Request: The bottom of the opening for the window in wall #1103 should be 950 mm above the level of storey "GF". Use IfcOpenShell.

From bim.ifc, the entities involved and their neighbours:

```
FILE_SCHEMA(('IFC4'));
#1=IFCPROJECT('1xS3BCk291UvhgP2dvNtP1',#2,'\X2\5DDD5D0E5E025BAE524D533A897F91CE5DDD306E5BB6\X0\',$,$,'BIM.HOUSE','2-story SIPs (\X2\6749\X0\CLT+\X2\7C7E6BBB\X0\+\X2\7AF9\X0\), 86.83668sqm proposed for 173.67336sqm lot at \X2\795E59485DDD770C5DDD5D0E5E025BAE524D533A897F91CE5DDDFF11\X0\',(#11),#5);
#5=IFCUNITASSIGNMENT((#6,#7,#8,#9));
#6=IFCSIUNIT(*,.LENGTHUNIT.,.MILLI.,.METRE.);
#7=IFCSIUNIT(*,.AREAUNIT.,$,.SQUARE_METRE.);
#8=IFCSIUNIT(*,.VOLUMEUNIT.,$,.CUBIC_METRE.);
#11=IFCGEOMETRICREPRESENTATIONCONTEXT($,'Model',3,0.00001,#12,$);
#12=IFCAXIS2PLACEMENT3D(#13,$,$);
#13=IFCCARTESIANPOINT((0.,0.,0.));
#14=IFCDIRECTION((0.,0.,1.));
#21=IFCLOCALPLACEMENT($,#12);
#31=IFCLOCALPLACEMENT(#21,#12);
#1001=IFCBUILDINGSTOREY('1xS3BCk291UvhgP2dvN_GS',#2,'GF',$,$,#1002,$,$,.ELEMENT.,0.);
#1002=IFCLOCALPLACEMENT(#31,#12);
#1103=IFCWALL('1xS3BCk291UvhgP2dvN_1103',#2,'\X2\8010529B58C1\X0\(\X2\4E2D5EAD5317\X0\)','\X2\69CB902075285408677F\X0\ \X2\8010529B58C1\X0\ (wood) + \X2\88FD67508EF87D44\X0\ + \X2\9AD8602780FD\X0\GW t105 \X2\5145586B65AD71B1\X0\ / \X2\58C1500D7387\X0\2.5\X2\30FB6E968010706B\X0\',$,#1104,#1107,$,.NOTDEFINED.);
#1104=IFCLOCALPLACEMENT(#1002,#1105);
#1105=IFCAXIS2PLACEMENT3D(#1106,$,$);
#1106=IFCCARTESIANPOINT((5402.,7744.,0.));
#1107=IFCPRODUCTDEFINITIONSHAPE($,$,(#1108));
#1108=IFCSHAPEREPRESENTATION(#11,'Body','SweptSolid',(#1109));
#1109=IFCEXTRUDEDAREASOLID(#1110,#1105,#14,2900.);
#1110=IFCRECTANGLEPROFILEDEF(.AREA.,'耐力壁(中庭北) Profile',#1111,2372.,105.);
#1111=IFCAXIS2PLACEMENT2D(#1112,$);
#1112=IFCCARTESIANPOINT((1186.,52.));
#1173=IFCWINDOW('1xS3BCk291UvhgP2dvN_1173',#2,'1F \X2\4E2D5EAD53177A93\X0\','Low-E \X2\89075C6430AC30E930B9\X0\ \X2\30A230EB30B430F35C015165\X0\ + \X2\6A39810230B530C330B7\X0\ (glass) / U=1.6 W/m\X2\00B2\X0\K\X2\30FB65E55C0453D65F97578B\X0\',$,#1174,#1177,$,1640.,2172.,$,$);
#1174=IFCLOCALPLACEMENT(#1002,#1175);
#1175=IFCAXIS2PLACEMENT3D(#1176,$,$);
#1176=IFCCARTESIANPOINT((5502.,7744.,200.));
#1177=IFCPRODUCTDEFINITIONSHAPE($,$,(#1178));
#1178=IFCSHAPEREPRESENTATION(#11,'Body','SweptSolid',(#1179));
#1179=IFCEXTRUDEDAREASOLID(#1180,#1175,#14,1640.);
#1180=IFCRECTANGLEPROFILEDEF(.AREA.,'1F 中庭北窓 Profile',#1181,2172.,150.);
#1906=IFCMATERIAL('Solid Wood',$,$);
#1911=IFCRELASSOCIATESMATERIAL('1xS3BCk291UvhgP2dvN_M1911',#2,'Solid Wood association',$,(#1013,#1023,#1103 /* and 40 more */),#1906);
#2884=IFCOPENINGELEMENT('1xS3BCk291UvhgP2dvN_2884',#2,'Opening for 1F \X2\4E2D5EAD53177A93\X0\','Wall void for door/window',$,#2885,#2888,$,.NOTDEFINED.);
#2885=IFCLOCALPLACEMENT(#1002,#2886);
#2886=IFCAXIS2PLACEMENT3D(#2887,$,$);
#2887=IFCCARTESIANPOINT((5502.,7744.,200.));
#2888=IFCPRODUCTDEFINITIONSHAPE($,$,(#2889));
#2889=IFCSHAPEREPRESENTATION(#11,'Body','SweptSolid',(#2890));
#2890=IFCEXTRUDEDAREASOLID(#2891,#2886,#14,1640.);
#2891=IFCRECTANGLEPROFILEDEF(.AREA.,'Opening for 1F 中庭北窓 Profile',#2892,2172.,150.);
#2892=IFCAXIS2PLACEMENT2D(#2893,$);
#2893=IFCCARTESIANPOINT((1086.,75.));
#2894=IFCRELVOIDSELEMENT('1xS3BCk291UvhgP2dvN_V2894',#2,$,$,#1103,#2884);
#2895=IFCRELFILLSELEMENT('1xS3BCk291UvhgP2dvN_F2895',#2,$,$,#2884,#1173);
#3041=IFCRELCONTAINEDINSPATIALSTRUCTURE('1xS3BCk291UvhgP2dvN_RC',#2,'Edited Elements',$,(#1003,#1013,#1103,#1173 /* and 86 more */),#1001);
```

```python
import numpy as np
import ifcopenshell
import ifcopenshell.api.geometry
import ifcopenshell.geom
import ifcopenshell.util.element
import ifcopenshell.util.placement
import ifcopenshell.util.shape
import ifcopenshell.util.unit

model = ifcopenshell.open("bim.ifc")
unit_scale = ifcopenshell.util.unit.calculate_unit_scale(model)

window = model.by_guid("1xS3BCk291UvhgP2dvN_1173")
opening = window.FillsVoids[0].RelatingOpeningElement
storey = ifcopenshell.util.element.get_container(window, ifc_class="IfcBuildingStorey")
level = ifcopenshell.util.placement.get_local_placement(storey.ObjectPlacement)[2, 3]

# The opening's origin need not be at the sill, so measure its lowest point.
shape = ifcopenshell.geom.create_shape(ifcopenshell.geom.settings(), opening)
bottom = ifcopenshell.util.shape.get_shape_bottom_elevation(shape, shape.geometry) / unit_scale
dz = level + 0.95 / unit_scale - bottom

shift = np.array([0.0, 0.0, dz])
# The window is not placed relative to its opening, so move both.
for product in (opening, window):
    matrix = ifcopenshell.util.placement.get_local_placement(product.ObjectPlacement)
    matrix[:3, 3] += shift
    ifcopenshell.api.geometry.edit_object_placement(model, product=product, matrix=matrix, is_si=False)

print(f"moved by {dz * unit_scale:+.3f} m")

model.write("bim_v2.ifc")
```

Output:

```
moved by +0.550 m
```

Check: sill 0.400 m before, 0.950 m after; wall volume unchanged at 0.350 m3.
